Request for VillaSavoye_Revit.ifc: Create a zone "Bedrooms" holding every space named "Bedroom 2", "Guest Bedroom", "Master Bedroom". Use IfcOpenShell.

First a look at what the model holds.

```python
import ifcopenshell

model = ifcopenshell.open("VillaSavoye_Revit.ifc")
print(model.schema)
seen = {}
for space in model.by_type("IfcSpace"):
    seen[space.LongName] = seen.get(space.LongName, 0) + 1
for name, count in sorted(seen.items(), key=str):
    print(count, "x", name)
print("zones:", [z.Name for z in model.by_type("IfcZone")][:20])
```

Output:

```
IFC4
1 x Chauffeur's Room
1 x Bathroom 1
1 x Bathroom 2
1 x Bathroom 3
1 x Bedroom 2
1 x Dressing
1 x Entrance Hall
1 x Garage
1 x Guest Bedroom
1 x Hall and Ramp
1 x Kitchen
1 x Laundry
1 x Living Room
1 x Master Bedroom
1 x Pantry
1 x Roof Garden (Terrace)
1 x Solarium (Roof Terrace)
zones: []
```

```python
import ifcopenshell
import ifcopenshell.api.group
import ifcopenshell.api.root

model = ifcopenshell.open("VillaSavoye_Revit.ifc")

names = {"Bedroom 2", "Guest Bedroom", "Master Bedroom"}
spaces = [s for s in model.by_type("IfcSpace") if s.LongName in names]

zone = ifcopenshell.api.root.create_entity(model, ifc_class="IfcZone", name="Bedrooms")
ifcopenshell.api.group.assign_group(model, products=spaces, group=zone)
print(len(spaces), "spaces in", zone.Name)

model.write("VillaSavoye_Revit_rev.ifc")
```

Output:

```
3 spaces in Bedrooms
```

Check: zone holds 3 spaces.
